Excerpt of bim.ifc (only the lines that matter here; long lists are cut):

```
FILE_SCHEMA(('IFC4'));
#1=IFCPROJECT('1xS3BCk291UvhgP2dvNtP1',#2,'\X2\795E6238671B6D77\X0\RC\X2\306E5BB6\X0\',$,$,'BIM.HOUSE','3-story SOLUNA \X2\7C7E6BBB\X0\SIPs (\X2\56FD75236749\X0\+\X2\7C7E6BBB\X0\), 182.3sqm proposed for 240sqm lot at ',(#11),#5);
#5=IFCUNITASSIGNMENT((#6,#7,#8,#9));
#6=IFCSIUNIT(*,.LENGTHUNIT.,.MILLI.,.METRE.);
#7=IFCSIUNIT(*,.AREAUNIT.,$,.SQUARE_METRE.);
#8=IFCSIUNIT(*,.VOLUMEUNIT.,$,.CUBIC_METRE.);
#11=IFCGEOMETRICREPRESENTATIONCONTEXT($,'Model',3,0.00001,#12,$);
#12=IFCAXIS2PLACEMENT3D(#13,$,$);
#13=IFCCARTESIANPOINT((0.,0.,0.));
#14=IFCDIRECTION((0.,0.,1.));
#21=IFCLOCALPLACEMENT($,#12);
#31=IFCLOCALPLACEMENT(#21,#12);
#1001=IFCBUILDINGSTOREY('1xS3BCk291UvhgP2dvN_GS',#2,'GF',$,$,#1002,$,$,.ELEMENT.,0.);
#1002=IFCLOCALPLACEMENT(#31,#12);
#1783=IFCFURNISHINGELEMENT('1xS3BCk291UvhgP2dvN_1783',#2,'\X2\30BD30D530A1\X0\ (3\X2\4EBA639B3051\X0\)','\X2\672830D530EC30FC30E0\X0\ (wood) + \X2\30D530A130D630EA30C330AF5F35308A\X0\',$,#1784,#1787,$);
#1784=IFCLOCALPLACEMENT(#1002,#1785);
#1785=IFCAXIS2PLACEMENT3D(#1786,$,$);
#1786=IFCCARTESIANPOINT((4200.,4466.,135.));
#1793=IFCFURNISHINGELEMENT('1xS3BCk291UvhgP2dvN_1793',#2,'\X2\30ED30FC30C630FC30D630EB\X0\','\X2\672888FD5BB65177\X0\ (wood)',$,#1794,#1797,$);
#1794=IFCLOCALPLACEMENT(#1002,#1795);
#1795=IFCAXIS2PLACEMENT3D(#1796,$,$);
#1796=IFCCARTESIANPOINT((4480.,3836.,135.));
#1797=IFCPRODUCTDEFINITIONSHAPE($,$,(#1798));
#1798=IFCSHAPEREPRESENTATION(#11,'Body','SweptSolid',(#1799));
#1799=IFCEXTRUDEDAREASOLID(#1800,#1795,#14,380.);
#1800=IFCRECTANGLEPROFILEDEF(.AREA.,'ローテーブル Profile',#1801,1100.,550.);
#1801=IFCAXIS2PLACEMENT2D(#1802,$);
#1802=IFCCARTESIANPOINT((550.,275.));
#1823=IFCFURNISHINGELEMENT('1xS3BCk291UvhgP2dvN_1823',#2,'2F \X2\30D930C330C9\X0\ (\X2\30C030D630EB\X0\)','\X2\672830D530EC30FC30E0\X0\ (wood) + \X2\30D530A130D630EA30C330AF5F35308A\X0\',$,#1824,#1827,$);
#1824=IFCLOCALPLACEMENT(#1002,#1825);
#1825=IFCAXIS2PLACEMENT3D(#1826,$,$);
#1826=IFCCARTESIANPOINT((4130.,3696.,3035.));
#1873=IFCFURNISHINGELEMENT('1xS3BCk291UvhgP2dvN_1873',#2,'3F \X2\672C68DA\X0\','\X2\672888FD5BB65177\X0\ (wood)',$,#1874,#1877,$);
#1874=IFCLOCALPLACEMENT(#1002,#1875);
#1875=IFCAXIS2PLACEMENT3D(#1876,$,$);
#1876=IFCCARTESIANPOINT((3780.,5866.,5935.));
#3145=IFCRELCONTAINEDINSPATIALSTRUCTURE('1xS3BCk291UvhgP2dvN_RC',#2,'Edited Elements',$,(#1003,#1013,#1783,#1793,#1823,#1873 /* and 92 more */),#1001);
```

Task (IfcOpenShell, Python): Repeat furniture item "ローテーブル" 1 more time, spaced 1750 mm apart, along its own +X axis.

```python
import ifcopenshell
import ifcopenshell.api.geometry
import ifcopenshell.api.root
import ifcopenshell.util.element
import ifcopenshell.util.placement
import ifcopenshell.util.unit

model = ifcopenshell.open("bim.ifc")
unit_scale = ifcopenshell.util.unit.calculate_unit_scale(model)


def reuse_history(source, copy):
    """copy_class also copies each property set's owner history, people and application; keep the originals."""
    for rel in copy.IsDefinedBy:
        if rel.is_a("IfcRelDefinesByProperties") and (history := rel.RelatingPropertyDefinition.OwnerHistory):
            rel.RelatingPropertyDefinition.OwnerHistory = source.OwnerHistory
            ifcopenshell.util.element.remove_deep2(model, history)


source = model.by_guid("1xS3BCk291UvhgP2dvN_1793")
base = ifcopenshell.util.placement.get_local_placement(source.ObjectPlacement)
step = base[:3, 0] * 1.75 / unit_scale

for i in range(1, 2):
    copy = ifcopenshell.api.root.copy_class(model, product=source)
    copy.Representation = ifcopenshell.util.element.copy_deep(
        model, source.Representation, exclude=["IfcGeometricRepresentationContext", "IfcRepresentationMap"]
    )
    reuse_history(source, copy)
    matrix = base.copy()
    matrix[:3, 3] += i * step
    print("added at", matrix[:3, 3].round(3) + 0.0)
    ifcopenshell.api.geometry.edit_object_placement(model, product=copy, matrix=matrix, is_si=False)

model.write("bim_edited.ifc")
```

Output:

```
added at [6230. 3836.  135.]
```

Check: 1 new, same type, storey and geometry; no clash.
